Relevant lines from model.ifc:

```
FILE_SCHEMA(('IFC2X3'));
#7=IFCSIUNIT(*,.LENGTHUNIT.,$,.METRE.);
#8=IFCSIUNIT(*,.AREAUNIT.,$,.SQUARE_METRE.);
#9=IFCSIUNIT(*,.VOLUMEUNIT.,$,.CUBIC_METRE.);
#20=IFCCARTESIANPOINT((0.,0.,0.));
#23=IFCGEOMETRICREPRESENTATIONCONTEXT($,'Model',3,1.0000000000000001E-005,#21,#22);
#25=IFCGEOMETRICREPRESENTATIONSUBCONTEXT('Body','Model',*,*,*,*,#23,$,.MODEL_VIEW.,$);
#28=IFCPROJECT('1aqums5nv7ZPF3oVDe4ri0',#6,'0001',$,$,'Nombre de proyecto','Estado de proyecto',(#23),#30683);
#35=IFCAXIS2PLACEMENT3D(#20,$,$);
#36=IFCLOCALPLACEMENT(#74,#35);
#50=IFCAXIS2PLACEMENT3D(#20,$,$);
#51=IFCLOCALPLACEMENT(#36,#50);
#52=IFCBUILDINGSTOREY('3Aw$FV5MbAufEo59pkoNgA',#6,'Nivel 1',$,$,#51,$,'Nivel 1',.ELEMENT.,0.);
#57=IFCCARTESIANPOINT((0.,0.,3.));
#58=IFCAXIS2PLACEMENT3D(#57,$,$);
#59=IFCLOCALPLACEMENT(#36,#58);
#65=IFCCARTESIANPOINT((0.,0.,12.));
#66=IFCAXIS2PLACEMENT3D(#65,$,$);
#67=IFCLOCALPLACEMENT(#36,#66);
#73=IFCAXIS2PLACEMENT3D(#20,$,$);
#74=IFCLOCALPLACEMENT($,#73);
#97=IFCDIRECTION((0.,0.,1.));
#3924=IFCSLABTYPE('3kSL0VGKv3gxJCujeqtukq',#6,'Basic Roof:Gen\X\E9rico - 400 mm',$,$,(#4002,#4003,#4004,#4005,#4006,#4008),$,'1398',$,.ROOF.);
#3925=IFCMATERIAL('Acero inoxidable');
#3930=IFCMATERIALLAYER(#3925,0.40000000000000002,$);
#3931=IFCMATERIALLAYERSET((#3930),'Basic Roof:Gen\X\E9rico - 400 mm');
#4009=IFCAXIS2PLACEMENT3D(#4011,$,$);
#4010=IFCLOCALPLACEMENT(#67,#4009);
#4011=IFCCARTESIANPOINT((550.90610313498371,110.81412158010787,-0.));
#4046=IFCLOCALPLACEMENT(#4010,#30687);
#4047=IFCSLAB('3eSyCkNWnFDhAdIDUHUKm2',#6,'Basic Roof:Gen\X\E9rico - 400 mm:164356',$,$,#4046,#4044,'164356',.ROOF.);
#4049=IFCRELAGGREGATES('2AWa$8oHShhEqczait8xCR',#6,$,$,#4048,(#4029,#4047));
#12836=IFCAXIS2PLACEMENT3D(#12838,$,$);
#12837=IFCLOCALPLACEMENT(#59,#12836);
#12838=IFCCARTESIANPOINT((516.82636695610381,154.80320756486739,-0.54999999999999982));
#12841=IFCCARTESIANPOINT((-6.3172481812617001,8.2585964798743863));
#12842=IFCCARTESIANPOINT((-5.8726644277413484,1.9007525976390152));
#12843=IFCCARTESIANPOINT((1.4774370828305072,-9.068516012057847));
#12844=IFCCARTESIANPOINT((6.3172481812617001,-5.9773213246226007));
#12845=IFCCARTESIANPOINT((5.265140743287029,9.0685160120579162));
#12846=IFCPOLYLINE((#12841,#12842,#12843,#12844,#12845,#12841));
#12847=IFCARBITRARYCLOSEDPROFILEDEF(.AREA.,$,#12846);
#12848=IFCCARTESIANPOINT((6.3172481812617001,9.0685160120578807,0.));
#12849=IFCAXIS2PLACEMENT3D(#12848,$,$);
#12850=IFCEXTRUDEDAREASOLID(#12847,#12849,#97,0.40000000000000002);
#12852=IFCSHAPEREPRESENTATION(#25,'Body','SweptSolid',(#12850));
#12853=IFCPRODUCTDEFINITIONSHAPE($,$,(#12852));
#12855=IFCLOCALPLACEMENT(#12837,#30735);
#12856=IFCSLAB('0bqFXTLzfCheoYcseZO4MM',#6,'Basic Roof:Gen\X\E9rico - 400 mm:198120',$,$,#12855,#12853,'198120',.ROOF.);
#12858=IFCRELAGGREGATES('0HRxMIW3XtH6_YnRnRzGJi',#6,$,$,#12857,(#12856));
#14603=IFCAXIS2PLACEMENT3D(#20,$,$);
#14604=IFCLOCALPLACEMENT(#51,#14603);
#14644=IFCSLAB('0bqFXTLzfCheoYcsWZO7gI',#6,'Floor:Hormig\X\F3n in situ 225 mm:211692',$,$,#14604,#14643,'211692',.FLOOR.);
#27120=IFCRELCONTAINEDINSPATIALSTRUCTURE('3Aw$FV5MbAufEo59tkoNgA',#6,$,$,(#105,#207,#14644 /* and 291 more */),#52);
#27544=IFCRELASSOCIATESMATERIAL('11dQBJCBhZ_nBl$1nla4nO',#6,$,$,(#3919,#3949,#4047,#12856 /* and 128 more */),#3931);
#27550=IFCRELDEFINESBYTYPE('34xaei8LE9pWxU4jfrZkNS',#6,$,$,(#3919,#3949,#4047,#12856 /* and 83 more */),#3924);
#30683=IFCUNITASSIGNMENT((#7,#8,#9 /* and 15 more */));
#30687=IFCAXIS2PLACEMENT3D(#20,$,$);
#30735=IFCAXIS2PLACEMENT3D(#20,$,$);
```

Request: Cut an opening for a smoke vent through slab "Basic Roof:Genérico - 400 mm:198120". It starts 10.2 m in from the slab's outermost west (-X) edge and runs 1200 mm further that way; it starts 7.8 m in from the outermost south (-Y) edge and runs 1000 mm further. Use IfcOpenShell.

```python
import numpy as np
import ifcopenshell
import ifcopenshell.api.feature
import ifcopenshell.api.geometry
import ifcopenshell.api.root
import ifcopenshell.geom
import ifcopenshell.util.placement
import ifcopenshell.util.representation
import ifcopenshell.util.shape
import ifcopenshell.util.unit

model = ifcopenshell.open("model.ifc")
unit_scale = ifcopenshell.util.unit.calculate_unit_scale(model)
settings = ifcopenshell.geom.settings()


def volume(element):
    """Net volume in cubic metres, openings subtracted."""
    shape = ifcopenshell.geom.create_shape(settings, element)
    return ifcopenshell.util.shape.get_volume(shape.geometry)


slab = model.by_guid("0bqFXTLzfCheoYcseZO4MM")
before = volume(slab)

# Extent in the slab's own axes, in metres. The edges named are its -X and -Y sides.
slab_shape = ifcopenshell.geom.create_shape(settings, slab)
vertices = ifcopenshell.util.shape.get_vertices(slab_shape.geometry)
x_min, y_min, bottom = vertices.min(axis=0)
top = vertices[:, 2].max()

opening = ifcopenshell.api.root.create_entity(model, ifc_class="IfcOpeningElement", name="Smoke vent opening")
context = ifcopenshell.util.representation.get_context(model, "Model", "Body", "MODEL_VIEW")
width, depth = 1.2, 1
outline = [(0.0, 0.0), (width, 0.0), (width, depth), (0.0, depth), (0.0, 0.0)]
# Overshoot both faces by 50 mm so the cut is clean.
shape = ifcopenshell.api.geometry.add_slab_representation(
    model, context=context, depth=top - bottom + 0.1, polyline=outline
)
ifcopenshell.api.geometry.assign_representation(model, product=opening, representation=shape)

matrix = ifcopenshell.util.placement.get_local_placement(slab.ObjectPlacement)
matrix[:, 3] = matrix @ np.append(np.array([x_min + 10.2, y_min + 7.8, bottom - 0.05]) / unit_scale, 1.0)
ifcopenshell.api.geometry.edit_object_placement(model, product=opening, matrix=matrix, is_si=False)
ifcopenshell.api.feature.add_feature(model, feature=opening, element=slab)

after = volume(slab)

print(f"slab volume {before:.3f} -> {after:.3f} m3")

model.write("model-out.ifc")
```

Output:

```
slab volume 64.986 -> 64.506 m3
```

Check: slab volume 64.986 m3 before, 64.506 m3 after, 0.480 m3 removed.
